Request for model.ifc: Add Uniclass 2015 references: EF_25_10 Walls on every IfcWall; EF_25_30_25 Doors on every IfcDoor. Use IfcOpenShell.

First a look at what the model holds.

```python
import ifcopenshell

model = ifcopenshell.open("model.ifc")
print(model.schema)
print("classifications:", [c.Name for c in model.by_type("IfcClassification")])
for ifc_class in ("IfcDoor", "IfcRoof", "IfcStair", "IfcWall", "IfcWindow"):
    print(ifc_class, len(model.by_type(ifc_class)))
```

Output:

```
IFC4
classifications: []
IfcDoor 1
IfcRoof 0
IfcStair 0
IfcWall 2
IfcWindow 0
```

```python
import ifcopenshell
import ifcopenshell.api.classification

model = ifcopenshell.open("model.ifc")

system = ifcopenshell.api.classification.add_classification(model, classification="Uniclass 2015")

codes = {
    "IfcWall": ("EF_25_10", "Walls"),
    "IfcDoor": ("EF_25_30_25", "Doors"),
}
for ifc_class, (code, name) in codes.items():
    products = model.by_type(ifc_class)
    ifcopenshell.api.classification.add_reference(
        model, products=products, classification=system, identification=code, name=name
    )
    print(code, len(products))

model.write("model_rev.ifc")
```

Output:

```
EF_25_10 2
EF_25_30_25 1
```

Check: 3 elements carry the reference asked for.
